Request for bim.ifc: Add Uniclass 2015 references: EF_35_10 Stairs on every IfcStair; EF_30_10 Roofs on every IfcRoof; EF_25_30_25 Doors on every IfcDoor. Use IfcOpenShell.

First a look at what the model holds.

```python
import ifcopenshell

model = ifcopenshell.open("bim.ifc")
print(model.schema)
print("classifications:", [c.Name for c in model.by_type("IfcClassification")])
for ifc_class in ("IfcDoor", "IfcRoof", "IfcStair", "IfcWall", "IfcWindow"):
    print(ifc_class, len(model.by_type(ifc_class)))
```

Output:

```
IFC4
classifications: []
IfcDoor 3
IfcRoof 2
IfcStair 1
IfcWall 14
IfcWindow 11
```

```python
import ifcopenshell
import ifcopenshell.api.classification

model = ifcopenshell.open("bim.ifc")

system = ifcopenshell.api.classification.add_classification(model, classification="Uniclass 2015")

codes = {
    "IfcStair": ("EF_35_10", "Stairs"),
    "IfcRoof": ("EF_30_10", "Roofs"),
    "IfcDoor": ("EF_25_30_25", "Doors"),
}
for ifc_class, (code, name) in codes.items():
    products = model.by_type(ifc_class)
    ifcopenshell.api.classification.add_reference(
        model, products=products, classification=system, identification=code, name=name
    )
    print(code, len(products))

model.write("bim_edited.ifc")
```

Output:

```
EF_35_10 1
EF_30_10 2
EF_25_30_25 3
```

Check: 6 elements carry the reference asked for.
